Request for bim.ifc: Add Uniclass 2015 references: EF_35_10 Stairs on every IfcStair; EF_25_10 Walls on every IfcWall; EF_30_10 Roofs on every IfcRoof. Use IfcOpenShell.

First a look at what the model holds.

```python
import ifcopenshell

model = ifcopenshell.open("bim.ifc")
print(model.schema)
print("classifications:", [c.Name for c in model.by_type("IfcClassification")])
for ifc_class in ("IfcDoor", "IfcRoof", "IfcStair", "IfcWall", "IfcWindow"):
    print(ifc_class, len(model.by_type(ifc_class)))
```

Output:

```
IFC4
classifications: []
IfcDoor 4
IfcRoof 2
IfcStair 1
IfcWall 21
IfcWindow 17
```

```python
import ifcopenshell
import ifcopenshell.api.classification

model = ifcopenshell.open("bim.ifc")

system = ifcopenshell.api.classification.add_classification(model, classification="Uniclass 2015")

codes = {
    "IfcStair": ("EF_35_10", "Stairs"),
    "IfcWall": ("EF_25_10", "Walls"),
    "IfcRoof": ("EF_30_10", "Roofs"),
}
for ifc_class, (code, name) in codes.items():
    products = model.by_type(ifc_class)
    ifcopenshell.api.classification.add_reference(
        model, products=products, classification=system, identification=code, name=name
    )
    print(code, len(products))

model.write("bim-out.ifc")
```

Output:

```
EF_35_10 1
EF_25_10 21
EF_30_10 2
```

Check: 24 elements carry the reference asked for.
